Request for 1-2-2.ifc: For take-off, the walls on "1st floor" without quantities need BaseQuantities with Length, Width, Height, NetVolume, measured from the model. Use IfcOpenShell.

First a look at what the model holds.

```python
import ifcopenshell
import ifcopenshell.util.element
import ifcopenshell.util.unit

model = ifcopenshell.open("1-2-2.ifc")
print(model.schema)
for unit_type in ("LENGTHUNIT", "AREAUNIT", "VOLUMEUNIT"):
    print(unit_type, ifcopenshell.util.unit.calculate_unit_scale(model, unit_type))
storey = next(s for s in model.by_type("IfcBuildingStorey") if s.Name == "1st floor")
walls = [e for e in ifcopenshell.util.element.get_decomposition(storey) if e.is_a("IfcWall")]
for e in sorted(walls, key=lambda e: e.id()):
    print(e.id(), e.is_a(), e.Name, list(ifcopenshell.util.element.get_psets(e, qtos_only=True)), sep=" | ")
```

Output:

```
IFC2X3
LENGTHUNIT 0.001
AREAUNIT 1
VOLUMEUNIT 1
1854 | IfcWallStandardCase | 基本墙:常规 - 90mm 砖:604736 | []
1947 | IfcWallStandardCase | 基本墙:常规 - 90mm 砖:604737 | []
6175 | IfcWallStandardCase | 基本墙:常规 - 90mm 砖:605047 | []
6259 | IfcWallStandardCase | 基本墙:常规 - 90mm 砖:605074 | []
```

```python
import ifcopenshell
import ifcopenshell.api.pset
import ifcopenshell.geom
import ifcopenshell.util.element
import ifcopenshell.util.shape
import ifcopenshell.util.unit

model = ifcopenshell.open("1-2-2.ifc")
unit_scale = ifcopenshell.util.unit.calculate_unit_scale(model)
volume_scale = ifcopenshell.util.unit.calculate_unit_scale(model, "VOLUMEUNIT")
settings = ifcopenshell.geom.settings()

storey = next(s for s in model.by_type("IfcBuildingStorey") if s.Name == "1st floor")
walls = [e for e in ifcopenshell.util.element.get_decomposition(storey) if e.is_a("IfcWall")]

for e in sorted(walls, key=lambda e: e.id()):
    if ifcopenshell.util.element.get_psets(e, qtos_only=True, should_inherit=False):
        continue
    # Geometry comes back in metres, in the element's own axes.
    shape = ifcopenshell.geom.create_shape(settings, e)
    values = {
        "Length": ifcopenshell.util.shape.get_x(shape.geometry) / unit_scale,
        "Width": ifcopenshell.util.shape.get_y(shape.geometry) / unit_scale,
        "Height": ifcopenshell.util.shape.get_z(shape.geometry) / unit_scale,
        "NetVolume": ifcopenshell.util.shape.get_volume(shape.geometry) / volume_scale,
    }
    qto = ifcopenshell.api.pset.add_qto(model, product=e, name="BaseQuantities")
    ifcopenshell.api.pset.edit_qto(model, qto=qto, properties=values)
    print(e.id(), {k: round(v, 3) for k, v in values.items()})

model.write("1-2-2_rev.ifc")
```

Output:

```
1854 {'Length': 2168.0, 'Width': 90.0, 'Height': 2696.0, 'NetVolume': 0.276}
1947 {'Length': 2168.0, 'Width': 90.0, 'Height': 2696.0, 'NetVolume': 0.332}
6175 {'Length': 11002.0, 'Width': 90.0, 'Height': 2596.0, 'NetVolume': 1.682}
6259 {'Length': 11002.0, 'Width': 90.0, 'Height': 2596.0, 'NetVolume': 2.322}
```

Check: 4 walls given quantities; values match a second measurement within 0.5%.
